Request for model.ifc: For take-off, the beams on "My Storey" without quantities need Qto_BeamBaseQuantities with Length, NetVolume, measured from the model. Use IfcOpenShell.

First a look at what the model holds.

```python
import ifcopenshell
import ifcopenshell.util.element
import ifcopenshell.util.unit

model = ifcopenshell.open("model.ifc")
print(model.schema)
for unit_type in ("LENGTHUNIT", "AREAUNIT", "VOLUMEUNIT"):
    print(unit_type, ifcopenshell.util.unit.calculate_unit_scale(model, unit_type))
storey = next(s for s in model.by_type("IfcBuildingStorey") if s.Name == "My Storey")
beams = [e for e in ifcopenshell.util.element.get_decomposition(storey) if e.is_a("IfcBeam")]
for e in sorted(beams, key=lambda e: e.id()):
    print(e.id(), e.is_a(), e.Name, list(ifcopenshell.util.element.get_psets(e, qtos_only=True)), sep=" | ")
```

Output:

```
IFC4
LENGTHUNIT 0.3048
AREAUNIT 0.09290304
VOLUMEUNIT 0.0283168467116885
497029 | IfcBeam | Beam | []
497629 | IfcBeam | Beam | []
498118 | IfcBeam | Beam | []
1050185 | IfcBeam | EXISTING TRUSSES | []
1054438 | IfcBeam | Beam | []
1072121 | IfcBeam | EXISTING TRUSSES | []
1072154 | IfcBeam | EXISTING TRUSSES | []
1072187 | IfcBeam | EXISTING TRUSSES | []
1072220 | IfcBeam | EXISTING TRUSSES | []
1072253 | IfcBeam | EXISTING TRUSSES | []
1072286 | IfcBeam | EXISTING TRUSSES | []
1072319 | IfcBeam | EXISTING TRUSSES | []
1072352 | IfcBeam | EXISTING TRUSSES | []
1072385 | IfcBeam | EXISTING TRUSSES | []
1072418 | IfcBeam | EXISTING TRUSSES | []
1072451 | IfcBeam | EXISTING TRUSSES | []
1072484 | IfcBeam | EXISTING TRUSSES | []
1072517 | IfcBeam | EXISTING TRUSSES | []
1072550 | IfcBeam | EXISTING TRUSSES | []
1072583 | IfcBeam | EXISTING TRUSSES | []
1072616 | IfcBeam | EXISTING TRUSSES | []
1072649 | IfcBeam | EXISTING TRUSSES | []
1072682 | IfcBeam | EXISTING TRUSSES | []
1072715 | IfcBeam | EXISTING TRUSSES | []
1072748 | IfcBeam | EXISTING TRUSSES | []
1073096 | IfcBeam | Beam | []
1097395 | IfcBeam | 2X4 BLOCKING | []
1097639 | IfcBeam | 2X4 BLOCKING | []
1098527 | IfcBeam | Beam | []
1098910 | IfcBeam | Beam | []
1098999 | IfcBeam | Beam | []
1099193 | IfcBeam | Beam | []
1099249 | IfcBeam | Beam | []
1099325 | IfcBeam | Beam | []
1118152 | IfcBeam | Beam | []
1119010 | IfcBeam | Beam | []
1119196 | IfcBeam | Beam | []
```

```python
import ifcopenshell
import ifcopenshell.api.pset
import ifcopenshell.geom
import ifcopenshell.util.element
import ifcopenshell.util.shape
import ifcopenshell.util.unit

model = ifcopenshell.open("model.ifc")
unit_scale = ifcopenshell.util.unit.calculate_unit_scale(model)
volume_scale = ifcopenshell.util.unit.calculate_unit_scale(model, "VOLUMEUNIT")
settings = ifcopenshell.geom.settings()

storey = next(s for s in model.by_type("IfcBuildingStorey") if s.Name == "My Storey")
beams = [e for e in ifcopenshell.util.element.get_decomposition(storey) if e.is_a("IfcBeam")]

for e in sorted(beams, key=lambda e: e.id()):
    if ifcopenshell.util.element.get_psets(e, qtos_only=True, should_inherit=False):
        continue
    # Geometry comes back in metres, in the element's own axes.
    shape = ifcopenshell.geom.create_shape(settings, e)
    values = {
        "Length": ifcopenshell.util.shape.get_max_xyz(shape.geometry) / unit_scale,
        "NetVolume": ifcopenshell.util.shape.get_volume(shape.geometry) / volume_scale,
    }
    qto = ifcopenshell.api.pset.add_qto(model, product=e, name="Qto_BeamBaseQuantities")
    ifcopenshell.api.pset.edit_qto(model, qto=qto, properties=values)
    print(e.id(), {k: round(v, 3) for k, v in values.items()})

model.write("model-out.ifc")
```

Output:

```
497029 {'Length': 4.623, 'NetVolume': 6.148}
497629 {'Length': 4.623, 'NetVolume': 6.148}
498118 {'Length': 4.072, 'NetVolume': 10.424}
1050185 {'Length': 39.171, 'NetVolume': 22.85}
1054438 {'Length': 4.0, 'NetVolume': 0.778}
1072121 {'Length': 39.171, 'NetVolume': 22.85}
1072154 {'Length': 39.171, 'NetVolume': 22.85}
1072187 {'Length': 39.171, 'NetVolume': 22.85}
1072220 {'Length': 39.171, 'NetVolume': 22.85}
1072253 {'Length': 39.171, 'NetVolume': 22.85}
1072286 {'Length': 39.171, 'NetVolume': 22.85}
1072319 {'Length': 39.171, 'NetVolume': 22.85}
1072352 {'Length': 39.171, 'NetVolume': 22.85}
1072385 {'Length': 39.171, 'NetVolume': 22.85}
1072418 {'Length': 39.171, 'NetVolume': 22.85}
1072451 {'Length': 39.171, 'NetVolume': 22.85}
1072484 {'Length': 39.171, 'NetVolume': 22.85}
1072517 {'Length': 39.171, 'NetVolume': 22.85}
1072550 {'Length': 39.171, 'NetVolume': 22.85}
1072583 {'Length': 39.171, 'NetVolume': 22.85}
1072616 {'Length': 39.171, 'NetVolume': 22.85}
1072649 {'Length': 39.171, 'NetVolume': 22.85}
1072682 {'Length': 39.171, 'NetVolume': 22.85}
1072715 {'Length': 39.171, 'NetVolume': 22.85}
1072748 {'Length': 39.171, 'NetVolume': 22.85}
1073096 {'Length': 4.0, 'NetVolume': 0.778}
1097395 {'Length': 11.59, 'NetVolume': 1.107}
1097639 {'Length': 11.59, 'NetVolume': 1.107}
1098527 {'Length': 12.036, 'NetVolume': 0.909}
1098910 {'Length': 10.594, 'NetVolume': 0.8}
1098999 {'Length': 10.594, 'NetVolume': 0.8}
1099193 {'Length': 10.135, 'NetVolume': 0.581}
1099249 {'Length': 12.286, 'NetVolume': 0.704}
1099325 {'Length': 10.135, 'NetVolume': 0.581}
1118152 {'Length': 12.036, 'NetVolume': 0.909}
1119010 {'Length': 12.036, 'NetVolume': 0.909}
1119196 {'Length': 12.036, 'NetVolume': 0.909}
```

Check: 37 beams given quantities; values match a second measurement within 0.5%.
